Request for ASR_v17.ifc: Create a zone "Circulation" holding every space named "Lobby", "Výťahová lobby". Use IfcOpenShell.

First a look at what the model holds.

```python
import ifcopenshell

model = ifcopenshell.open("ASR_v17.ifc")
print(model.schema)
seen = {}
for space in model.by_type("IfcSpace"):
    seen[space.LongName] = seen.get(space.LongName, 0) + 1
for name, count in sorted(seen.items(), key=str):
    print(count, "x", name)
print("zones:", [z.Name for z in model.by_type("IfcZone")][:20])
```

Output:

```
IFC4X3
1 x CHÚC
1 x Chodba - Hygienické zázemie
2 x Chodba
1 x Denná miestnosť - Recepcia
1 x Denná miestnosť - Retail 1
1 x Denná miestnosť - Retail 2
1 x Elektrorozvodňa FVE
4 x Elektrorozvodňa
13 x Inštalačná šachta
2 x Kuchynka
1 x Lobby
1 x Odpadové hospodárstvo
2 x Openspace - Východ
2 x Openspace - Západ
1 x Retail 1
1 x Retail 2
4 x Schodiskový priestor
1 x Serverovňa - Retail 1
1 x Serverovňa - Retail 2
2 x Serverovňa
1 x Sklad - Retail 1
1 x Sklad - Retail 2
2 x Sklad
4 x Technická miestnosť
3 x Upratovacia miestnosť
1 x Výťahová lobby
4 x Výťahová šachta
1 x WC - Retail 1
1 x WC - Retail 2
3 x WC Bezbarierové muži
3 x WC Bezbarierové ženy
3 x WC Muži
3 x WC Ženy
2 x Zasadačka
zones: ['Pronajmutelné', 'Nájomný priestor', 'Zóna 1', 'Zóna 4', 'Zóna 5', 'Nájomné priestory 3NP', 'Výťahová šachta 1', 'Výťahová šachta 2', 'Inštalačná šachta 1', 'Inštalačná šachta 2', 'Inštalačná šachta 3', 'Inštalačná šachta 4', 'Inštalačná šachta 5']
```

```python
import ifcopenshell
import ifcopenshell.api.group
import ifcopenshell.api.root

model = ifcopenshell.open("ASR_v17.ifc")

names = {"Lobby", "Výťahová lobby"}
spaces = [s for s in model.by_type("IfcSpace") if s.LongName in names]

zone = ifcopenshell.api.root.create_entity(model, ifc_class="IfcZone", name="Circulation")
ifcopenshell.api.group.assign_group(model, products=spaces, group=zone)
print(len(spaces), "spaces in", zone.Name)

model.write("ASR_v17_v2.ifc")
```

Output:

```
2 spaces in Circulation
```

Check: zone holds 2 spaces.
